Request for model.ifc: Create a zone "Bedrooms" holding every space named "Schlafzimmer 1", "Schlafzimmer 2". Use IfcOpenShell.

First a look at what the model holds.

```python
import ifcopenshell

model = ifcopenshell.open("model.ifc")
print(model.schema)
seen = {}
for space in model.by_type("IfcSpace"):
    seen[space.LongName] = seen.get(space.LongName, 0) + 1
for name, count in sorted(seen.items(), key=str):
    print(count, "x", name)
print("zones:", [z.Name for z in model.by_type("IfcZone")][:20])
```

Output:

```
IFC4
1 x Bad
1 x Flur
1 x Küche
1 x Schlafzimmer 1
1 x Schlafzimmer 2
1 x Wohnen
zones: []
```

```python
import ifcopenshell
import ifcopenshell.api.group
import ifcopenshell.api.root

model = ifcopenshell.open("model.ifc")

names = {"Schlafzimmer 1", "Schlafzimmer 2"}
spaces = [s for s in model.by_type("IfcSpace") if s.LongName in names]

zone = ifcopenshell.api.root.create_entity(model, ifc_class="IfcZone", name="Bedrooms")
ifcopenshell.api.group.assign_group(model, products=spaces, group=zone)
print(len(spaces), "spaces in", zone.Name)

model.write("model_edited.ifc")
```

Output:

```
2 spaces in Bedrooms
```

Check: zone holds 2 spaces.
